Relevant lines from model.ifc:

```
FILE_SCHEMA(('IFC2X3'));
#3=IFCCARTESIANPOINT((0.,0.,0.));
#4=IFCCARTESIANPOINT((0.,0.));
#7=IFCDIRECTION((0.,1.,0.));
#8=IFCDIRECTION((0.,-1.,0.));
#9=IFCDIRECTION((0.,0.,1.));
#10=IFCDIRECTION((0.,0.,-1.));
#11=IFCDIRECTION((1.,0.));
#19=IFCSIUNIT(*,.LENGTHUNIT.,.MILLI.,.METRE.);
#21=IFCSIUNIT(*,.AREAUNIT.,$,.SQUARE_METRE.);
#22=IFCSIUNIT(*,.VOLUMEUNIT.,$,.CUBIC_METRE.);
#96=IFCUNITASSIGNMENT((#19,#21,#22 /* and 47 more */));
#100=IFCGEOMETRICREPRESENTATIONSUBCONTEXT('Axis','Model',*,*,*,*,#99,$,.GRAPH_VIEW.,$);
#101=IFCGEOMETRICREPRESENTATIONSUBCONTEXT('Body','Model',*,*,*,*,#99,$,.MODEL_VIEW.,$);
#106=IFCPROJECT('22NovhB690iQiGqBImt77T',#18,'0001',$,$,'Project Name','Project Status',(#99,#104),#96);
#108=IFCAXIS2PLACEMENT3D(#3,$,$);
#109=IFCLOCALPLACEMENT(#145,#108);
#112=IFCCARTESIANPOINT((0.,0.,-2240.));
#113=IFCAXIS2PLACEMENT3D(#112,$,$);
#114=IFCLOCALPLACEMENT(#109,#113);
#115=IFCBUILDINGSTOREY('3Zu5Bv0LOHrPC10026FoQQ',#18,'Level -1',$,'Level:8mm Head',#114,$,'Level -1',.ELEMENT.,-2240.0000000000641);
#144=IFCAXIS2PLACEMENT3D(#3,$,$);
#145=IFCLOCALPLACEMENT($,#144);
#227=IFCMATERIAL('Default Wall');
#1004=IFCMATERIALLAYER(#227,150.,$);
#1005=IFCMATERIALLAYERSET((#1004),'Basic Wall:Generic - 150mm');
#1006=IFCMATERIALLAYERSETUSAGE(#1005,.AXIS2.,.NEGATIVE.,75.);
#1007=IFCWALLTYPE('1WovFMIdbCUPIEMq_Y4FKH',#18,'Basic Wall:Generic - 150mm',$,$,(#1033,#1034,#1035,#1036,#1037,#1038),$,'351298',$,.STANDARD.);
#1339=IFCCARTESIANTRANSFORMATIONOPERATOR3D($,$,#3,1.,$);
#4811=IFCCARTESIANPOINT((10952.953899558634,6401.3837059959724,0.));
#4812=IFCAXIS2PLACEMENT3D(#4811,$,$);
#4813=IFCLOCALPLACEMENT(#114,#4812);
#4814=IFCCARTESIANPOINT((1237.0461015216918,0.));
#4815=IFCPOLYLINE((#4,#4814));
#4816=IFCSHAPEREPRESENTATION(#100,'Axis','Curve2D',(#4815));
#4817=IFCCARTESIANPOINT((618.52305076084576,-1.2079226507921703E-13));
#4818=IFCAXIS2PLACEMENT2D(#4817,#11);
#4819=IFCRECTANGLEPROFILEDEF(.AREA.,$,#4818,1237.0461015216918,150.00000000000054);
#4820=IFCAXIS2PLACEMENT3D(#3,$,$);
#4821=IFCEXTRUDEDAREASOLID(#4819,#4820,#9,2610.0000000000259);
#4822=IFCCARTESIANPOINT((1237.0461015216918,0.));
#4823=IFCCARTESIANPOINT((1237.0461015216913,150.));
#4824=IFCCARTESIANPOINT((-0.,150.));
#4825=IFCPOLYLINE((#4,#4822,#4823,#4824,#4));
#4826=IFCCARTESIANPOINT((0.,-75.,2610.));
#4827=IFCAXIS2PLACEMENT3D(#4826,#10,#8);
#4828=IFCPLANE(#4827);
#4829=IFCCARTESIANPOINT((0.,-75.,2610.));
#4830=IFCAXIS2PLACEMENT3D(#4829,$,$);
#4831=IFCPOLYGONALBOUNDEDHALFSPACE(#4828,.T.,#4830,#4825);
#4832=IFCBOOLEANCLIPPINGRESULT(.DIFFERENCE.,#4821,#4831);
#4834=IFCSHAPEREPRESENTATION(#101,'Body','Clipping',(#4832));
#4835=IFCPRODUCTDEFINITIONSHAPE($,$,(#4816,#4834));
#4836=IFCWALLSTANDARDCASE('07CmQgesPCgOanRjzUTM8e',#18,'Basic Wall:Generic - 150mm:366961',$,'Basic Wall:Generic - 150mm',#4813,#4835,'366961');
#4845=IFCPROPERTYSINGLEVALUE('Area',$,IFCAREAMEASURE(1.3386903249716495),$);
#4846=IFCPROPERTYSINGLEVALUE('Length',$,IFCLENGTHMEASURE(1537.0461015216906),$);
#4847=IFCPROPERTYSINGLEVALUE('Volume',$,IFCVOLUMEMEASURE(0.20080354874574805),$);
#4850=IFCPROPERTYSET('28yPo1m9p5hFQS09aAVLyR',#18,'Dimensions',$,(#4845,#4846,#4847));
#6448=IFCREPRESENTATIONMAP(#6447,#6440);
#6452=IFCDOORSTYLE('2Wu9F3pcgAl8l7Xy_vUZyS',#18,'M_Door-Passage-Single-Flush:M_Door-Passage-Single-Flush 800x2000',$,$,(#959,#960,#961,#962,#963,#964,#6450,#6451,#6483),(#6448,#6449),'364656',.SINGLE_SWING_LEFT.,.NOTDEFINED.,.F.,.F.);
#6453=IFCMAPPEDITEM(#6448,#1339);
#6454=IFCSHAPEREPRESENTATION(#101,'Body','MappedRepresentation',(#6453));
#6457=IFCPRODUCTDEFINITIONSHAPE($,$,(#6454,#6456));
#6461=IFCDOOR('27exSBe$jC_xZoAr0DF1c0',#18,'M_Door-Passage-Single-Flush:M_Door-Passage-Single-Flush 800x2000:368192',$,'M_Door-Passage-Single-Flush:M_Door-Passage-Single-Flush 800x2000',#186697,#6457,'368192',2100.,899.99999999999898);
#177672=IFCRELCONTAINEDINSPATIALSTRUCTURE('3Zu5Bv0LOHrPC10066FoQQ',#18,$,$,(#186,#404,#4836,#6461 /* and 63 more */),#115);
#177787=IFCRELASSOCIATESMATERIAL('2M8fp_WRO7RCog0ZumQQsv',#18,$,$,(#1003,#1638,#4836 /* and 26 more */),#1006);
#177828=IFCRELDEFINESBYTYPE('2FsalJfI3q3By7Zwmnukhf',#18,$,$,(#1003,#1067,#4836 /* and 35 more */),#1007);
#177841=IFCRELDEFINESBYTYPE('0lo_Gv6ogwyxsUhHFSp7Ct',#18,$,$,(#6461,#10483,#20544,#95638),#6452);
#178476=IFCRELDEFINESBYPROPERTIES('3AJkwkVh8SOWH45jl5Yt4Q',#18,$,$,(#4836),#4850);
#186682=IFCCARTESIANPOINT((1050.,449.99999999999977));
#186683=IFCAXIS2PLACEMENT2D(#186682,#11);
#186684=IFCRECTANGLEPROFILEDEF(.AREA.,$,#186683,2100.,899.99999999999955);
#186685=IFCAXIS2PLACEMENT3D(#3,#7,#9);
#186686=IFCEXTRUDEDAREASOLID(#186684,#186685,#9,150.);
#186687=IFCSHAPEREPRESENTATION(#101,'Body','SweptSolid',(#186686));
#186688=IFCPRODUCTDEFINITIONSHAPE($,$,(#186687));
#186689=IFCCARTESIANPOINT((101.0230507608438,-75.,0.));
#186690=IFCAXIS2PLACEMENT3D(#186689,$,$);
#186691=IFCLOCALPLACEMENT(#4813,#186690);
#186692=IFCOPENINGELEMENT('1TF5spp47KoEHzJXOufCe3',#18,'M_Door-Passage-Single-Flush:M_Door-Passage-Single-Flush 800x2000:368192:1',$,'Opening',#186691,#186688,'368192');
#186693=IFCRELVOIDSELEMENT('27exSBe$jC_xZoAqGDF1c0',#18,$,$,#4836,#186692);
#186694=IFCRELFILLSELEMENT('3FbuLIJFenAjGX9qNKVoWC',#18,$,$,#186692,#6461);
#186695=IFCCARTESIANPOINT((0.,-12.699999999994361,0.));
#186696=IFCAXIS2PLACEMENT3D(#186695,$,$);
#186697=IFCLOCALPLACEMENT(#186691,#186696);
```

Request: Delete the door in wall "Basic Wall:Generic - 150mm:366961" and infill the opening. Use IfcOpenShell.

```python
import ifcopenshell
import ifcopenshell.api.feature
import ifcopenshell.api.pset
import ifcopenshell.api.root
import ifcopenshell.geom
import ifcopenshell.util.element
import ifcopenshell.util.shape
import ifcopenshell.util.unit

model = ifcopenshell.open("model.ifc")
area_scale = ifcopenshell.util.unit.calculate_unit_scale(model, "AREAUNIT")
volume_scale = ifcopenshell.util.unit.calculate_unit_scale(model, "VOLUMEUNIT")
settings = ifcopenshell.geom.settings()


def volume(element):
    """Net volume in cubic metres, openings subtracted."""
    shape = ifcopenshell.geom.create_shape(settings, element)
    return ifcopenshell.util.shape.get_volume(shape.geometry)


door = model.by_guid("27exSBe$jC_xZoAr0DF1c0")
opening = door.FillsVoids[0].RelatingOpeningElement
wall = opening.VoidsElements[0].RelatingBuildingElement
before = volume(wall)

ifcopenshell.api.root.remove_product(model, product=door)
ifcopenshell.api.feature.remove_feature(model, feature=opening)

after = volume(wall)
thickness = 0.15  # wall thickness in metres

# Update the wall's stored quantities.
pset = model.by_id(ifcopenshell.util.element.get_pset(wall, "Dimensions", should_inherit=False)["id"])
ifcopenshell.api.pset.edit_pset(model, pset=pset, properties={
    "Area": model.create_entity("IfcAreaMeasure", after / thickness / area_scale),
    "Volume": model.create_entity("IfcVolumeMeasure", after / volume_scale),
})

print(f"wall volume {before:.3f} -> {after:.3f} m3")

model.write("model_v2.ifc")
```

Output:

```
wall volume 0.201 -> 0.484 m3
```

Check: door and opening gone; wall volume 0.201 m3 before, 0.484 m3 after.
